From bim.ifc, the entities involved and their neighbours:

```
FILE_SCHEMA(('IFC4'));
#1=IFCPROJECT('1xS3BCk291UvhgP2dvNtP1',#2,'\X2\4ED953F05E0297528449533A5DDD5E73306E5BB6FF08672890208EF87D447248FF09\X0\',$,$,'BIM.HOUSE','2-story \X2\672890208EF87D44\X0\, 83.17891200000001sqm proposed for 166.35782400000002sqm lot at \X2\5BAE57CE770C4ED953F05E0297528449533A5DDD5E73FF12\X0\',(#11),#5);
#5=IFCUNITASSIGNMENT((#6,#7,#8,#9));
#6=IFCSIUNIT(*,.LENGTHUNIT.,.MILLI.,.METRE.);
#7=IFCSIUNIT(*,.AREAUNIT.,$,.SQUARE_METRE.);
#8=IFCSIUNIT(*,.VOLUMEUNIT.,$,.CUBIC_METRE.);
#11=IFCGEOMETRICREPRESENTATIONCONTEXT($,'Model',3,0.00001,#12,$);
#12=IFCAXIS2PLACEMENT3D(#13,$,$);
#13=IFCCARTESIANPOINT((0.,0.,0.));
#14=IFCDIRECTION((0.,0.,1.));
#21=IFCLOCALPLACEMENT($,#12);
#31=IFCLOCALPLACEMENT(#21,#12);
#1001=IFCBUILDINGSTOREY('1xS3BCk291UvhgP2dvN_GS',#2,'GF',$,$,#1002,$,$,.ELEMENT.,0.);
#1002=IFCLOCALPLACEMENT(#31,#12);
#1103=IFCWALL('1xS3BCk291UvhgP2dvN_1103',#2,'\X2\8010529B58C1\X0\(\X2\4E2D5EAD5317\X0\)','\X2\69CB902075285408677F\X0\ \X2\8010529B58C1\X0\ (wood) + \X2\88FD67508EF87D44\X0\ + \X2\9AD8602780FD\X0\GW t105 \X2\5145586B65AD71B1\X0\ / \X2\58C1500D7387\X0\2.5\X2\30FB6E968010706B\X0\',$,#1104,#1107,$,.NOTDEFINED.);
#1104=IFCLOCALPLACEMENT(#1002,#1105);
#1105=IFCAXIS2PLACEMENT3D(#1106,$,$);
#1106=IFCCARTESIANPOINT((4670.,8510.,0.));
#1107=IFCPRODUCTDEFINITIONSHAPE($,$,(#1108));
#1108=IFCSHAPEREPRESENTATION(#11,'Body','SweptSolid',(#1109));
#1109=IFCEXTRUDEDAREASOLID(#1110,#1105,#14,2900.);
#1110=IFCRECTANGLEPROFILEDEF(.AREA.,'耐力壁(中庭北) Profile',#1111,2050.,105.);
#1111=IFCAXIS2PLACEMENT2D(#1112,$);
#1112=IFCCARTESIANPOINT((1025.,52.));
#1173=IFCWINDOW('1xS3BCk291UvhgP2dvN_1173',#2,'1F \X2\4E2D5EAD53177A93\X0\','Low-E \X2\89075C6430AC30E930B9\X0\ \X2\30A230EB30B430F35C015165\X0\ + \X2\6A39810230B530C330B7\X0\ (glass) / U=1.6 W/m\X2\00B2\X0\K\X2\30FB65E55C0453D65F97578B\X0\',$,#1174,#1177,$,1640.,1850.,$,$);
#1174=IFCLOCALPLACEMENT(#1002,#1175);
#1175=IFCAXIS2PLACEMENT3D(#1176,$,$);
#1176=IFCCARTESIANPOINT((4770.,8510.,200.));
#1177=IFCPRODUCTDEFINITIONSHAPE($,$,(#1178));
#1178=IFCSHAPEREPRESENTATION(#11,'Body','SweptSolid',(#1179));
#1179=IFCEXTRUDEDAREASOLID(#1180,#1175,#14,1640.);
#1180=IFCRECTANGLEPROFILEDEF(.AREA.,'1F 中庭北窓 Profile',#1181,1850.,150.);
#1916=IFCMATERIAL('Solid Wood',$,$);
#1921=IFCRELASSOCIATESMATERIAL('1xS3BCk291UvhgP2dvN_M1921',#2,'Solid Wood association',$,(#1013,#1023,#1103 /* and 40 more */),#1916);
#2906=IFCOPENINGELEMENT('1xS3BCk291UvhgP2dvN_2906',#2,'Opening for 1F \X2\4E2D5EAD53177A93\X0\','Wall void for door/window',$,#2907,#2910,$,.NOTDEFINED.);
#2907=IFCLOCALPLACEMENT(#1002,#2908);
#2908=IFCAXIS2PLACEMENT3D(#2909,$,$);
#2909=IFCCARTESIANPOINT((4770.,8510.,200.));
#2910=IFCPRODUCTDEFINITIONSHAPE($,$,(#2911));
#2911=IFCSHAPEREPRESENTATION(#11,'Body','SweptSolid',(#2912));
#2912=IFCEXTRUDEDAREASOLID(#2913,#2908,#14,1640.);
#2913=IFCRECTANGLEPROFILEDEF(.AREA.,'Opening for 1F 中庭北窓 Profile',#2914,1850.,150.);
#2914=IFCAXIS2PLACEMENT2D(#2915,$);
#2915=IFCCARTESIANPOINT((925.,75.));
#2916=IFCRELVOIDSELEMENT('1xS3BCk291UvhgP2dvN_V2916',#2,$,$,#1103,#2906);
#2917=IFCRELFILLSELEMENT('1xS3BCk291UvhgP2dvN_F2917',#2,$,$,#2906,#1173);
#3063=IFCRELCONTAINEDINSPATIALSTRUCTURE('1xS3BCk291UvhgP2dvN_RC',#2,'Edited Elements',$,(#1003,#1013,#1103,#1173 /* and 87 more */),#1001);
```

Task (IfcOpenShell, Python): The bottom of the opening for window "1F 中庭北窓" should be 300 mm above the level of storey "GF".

```python
import numpy as np
import ifcopenshell
import ifcopenshell.api.geometry
import ifcopenshell.geom
import ifcopenshell.util.element
import ifcopenshell.util.placement
import ifcopenshell.util.shape
import ifcopenshell.util.unit

model = ifcopenshell.open("bim.ifc")
unit_scale = ifcopenshell.util.unit.calculate_unit_scale(model)

window = model.by_guid("1xS3BCk291UvhgP2dvN_1173")
opening = window.FillsVoids[0].RelatingOpeningElement
storey = ifcopenshell.util.element.get_container(window, ifc_class="IfcBuildingStorey")
level = ifcopenshell.util.placement.get_local_placement(storey.ObjectPlacement)[2, 3]

# The opening's origin need not be at the sill, so measure its lowest point.
shape = ifcopenshell.geom.create_shape(ifcopenshell.geom.settings(), opening)
bottom = ifcopenshell.util.shape.get_shape_bottom_elevation(shape, shape.geometry) / unit_scale
dz = level + 0.3 / unit_scale - bottom

shift = np.array([0.0, 0.0, dz])
# The window is not placed relative to its opening, so move both.
for product in (opening, window):
    matrix = ifcopenshell.util.placement.get_local_placement(product.ObjectPlacement)
    matrix[:3, 3] += shift
    ifcopenshell.api.geometry.edit_object_placement(model, product=product, matrix=matrix, is_si=False)

print(f"moved by {dz * unit_scale:+.3f} m")

model.write("bim_rev.ifc")
```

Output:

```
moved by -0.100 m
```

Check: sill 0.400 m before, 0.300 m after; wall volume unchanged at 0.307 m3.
